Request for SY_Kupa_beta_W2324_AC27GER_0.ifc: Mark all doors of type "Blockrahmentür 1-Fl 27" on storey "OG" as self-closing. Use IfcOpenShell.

First a look at what the model holds.

```python
import ifcopenshell
import ifcopenshell.util.element

model = ifcopenshell.open("SY_Kupa_beta_W2324_AC27GER_0.ifc")
print(model.schema)
storey = next(s for s in model.by_type("IfcBuildingStorey") if s.Name == "OG")
doors = [e for e in ifcopenshell.util.element.get_decomposition(storey) if e.is_a("IfcDoor")]
seen = {}
for e in doors:
    element_type = ifcopenshell.util.element.get_type(e)
    key = (element_type.Name if element_type != e and element_type else None, ifcopenshell.util.element.get_pset(e, "Pset_DoorCommon", "SelfClosing"))
    seen[key] = seen.get(key, 0) + 1
for (name, value), count in sorted(seen.items(), key=str):
    print(count, "x", name, "|", value)
```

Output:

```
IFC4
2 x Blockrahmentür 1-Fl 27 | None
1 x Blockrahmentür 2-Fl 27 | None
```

```python
import ifcopenshell
import ifcopenshell.api.pset
import ifcopenshell.util.element

model = ifcopenshell.open("SY_Kupa_beta_W2324_AC27GER_0.ifc")

storey = next(s for s in model.by_type("IfcBuildingStorey") if s.Name == "OG")
doors = [e for e in ifcopenshell.util.element.get_decomposition(storey) if e.is_a("IfcDoor")]

count = 0
for e in doors:
    element_type = ifcopenshell.util.element.get_type(e)
    if element_type in (None, e) or element_type.Name != "Blockrahmentür 1-Fl 27":
        continue
    # add_pset returns the element's existing set when there is one.
    pset = ifcopenshell.api.pset.add_pset(model, product=e, name="Pset_DoorCommon")
    ifcopenshell.api.pset.edit_pset(model, pset=pset, properties={"SelfClosing": True})
    count += 1

print(count, "doors updated")

model.write("SY_Kupa_beta_W2324_AC27GER_0_edited.ifc")
```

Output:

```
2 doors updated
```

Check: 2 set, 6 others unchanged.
